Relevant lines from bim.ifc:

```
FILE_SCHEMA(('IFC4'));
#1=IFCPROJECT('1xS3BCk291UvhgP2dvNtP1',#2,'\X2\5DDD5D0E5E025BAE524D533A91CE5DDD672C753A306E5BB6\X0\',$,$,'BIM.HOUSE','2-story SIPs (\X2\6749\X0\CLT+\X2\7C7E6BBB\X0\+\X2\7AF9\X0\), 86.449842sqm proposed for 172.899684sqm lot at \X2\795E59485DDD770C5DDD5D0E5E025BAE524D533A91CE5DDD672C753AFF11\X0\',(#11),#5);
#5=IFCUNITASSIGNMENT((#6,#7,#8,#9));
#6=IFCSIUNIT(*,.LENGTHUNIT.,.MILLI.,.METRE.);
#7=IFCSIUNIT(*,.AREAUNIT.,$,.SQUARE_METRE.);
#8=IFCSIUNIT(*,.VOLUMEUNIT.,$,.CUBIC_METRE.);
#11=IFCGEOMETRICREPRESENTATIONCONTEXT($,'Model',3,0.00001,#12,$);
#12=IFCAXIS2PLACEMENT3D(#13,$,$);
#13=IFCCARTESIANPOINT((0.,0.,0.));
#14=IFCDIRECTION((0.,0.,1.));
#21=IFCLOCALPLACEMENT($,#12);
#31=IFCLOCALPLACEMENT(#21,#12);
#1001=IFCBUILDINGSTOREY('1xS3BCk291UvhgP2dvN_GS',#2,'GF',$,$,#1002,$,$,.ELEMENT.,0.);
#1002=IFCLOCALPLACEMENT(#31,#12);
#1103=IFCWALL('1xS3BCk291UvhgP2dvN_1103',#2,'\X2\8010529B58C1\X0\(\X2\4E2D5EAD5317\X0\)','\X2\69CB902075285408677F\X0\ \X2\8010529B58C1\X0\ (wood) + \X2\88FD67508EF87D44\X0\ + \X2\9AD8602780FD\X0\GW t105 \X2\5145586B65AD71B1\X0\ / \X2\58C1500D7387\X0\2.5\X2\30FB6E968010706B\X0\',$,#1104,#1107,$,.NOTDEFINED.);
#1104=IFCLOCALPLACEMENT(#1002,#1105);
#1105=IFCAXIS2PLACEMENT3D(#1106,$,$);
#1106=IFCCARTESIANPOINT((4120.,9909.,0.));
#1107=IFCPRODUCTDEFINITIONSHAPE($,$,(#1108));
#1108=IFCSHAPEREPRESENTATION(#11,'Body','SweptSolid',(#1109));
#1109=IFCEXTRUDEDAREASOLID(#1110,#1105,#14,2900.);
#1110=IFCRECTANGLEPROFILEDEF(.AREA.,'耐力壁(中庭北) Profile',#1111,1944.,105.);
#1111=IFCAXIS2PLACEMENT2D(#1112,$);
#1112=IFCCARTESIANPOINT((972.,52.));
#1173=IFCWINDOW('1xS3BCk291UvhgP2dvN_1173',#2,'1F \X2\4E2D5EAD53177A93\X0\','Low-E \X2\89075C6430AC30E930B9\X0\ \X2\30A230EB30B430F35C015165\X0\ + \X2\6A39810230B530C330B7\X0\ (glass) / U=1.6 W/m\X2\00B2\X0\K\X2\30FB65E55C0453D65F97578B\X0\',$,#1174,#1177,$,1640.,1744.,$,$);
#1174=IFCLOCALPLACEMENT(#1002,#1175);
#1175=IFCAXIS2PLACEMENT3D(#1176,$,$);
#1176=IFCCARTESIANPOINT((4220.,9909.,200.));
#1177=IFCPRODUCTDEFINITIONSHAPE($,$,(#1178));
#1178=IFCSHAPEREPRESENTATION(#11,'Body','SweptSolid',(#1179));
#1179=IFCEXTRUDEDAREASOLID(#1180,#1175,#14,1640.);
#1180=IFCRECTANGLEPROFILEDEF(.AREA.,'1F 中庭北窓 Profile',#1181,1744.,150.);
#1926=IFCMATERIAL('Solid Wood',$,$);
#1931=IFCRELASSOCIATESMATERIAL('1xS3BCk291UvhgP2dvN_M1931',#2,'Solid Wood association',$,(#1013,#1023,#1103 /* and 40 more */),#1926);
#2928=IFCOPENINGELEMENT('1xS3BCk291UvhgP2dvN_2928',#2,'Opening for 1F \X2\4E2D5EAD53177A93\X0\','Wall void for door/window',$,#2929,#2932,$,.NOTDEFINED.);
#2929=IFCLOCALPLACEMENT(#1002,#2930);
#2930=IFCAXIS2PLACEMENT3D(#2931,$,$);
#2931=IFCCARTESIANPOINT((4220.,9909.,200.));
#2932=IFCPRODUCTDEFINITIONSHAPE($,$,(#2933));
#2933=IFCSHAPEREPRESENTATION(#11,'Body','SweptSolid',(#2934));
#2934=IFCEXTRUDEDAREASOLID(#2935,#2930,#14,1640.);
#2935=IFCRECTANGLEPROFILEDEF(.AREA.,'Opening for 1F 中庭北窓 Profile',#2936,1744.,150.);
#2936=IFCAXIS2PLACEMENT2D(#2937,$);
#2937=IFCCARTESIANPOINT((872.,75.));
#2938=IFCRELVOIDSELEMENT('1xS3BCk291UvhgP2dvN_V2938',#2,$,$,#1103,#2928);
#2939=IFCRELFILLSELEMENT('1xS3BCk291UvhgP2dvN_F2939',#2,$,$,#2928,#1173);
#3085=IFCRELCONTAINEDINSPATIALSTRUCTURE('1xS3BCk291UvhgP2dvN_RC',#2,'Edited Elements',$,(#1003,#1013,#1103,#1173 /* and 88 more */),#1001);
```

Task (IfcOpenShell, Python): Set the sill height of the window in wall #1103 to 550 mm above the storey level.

```python
import numpy as np
import ifcopenshell
import ifcopenshell.api.geometry
import ifcopenshell.geom
import ifcopenshell.util.element
import ifcopenshell.util.placement
import ifcopenshell.util.shape
import ifcopenshell.util.unit

model = ifcopenshell.open("bim.ifc")
unit_scale = ifcopenshell.util.unit.calculate_unit_scale(model)

window = model.by_id(1173)
opening = window.FillsVoids[0].RelatingOpeningElement
storey = ifcopenshell.util.element.get_container(window, ifc_class="IfcBuildingStorey")
level = ifcopenshell.util.placement.get_local_placement(storey.ObjectPlacement)[2, 3]

# The opening's origin need not be at the sill, so measure its lowest point.
shape = ifcopenshell.geom.create_shape(ifcopenshell.geom.settings(), opening)
bottom = ifcopenshell.util.shape.get_shape_bottom_elevation(shape, shape.geometry) / unit_scale
dz = level + 550.0 - bottom

shift = np.array([0.0, 0.0, dz])
# The window is not placed relative to its opening, so move both.
for product in (opening, window):
    matrix = ifcopenshell.util.placement.get_local_placement(product.ObjectPlacement)
    matrix[:3, 3] += shift
    ifcopenshell.api.geometry.edit_object_placement(model, product=product, matrix=matrix, is_si=False)

print(f"moved by {dz * unit_scale:+.3f} m")

model.write("bim_edited.ifc")
```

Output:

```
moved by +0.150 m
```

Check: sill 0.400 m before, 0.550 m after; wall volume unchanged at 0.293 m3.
